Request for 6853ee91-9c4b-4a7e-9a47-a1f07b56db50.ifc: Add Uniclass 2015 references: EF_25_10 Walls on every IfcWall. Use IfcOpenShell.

First a look at what the model holds.

```python
import ifcopenshell

model = ifcopenshell.open("6853ee91-9c4b-4a7e-9a47-a1f07b56db50.ifc")
print(model.schema)
print("classifications:", [c.Name for c in model.by_type("IfcClassification")])
for ifc_class in ("IfcDoor", "IfcRoof", "IfcStair", "IfcWall", "IfcWindow"):
    print(ifc_class, len(model.by_type(ifc_class)))
```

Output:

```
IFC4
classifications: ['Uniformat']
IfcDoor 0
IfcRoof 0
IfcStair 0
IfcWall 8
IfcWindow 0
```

```python
import ifcopenshell
import ifcopenshell.api.classification

model = ifcopenshell.open("6853ee91-9c4b-4a7e-9a47-a1f07b56db50.ifc")

system = ifcopenshell.api.classification.add_classification(model, classification="Uniclass 2015")

codes = {
    "IfcWall": ("EF_25_10", "Walls"),
}
for ifc_class, (code, name) in codes.items():
    products = model.by_type(ifc_class)
    ifcopenshell.api.classification.add_reference(
        model, products=products, classification=system, identification=code, name=name
    )
    print(code, len(products))

model.write("6853ee91-9c4b-4a7e-9a47-a1f07b56db50_updated.ifc")
```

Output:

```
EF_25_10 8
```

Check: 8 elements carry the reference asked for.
